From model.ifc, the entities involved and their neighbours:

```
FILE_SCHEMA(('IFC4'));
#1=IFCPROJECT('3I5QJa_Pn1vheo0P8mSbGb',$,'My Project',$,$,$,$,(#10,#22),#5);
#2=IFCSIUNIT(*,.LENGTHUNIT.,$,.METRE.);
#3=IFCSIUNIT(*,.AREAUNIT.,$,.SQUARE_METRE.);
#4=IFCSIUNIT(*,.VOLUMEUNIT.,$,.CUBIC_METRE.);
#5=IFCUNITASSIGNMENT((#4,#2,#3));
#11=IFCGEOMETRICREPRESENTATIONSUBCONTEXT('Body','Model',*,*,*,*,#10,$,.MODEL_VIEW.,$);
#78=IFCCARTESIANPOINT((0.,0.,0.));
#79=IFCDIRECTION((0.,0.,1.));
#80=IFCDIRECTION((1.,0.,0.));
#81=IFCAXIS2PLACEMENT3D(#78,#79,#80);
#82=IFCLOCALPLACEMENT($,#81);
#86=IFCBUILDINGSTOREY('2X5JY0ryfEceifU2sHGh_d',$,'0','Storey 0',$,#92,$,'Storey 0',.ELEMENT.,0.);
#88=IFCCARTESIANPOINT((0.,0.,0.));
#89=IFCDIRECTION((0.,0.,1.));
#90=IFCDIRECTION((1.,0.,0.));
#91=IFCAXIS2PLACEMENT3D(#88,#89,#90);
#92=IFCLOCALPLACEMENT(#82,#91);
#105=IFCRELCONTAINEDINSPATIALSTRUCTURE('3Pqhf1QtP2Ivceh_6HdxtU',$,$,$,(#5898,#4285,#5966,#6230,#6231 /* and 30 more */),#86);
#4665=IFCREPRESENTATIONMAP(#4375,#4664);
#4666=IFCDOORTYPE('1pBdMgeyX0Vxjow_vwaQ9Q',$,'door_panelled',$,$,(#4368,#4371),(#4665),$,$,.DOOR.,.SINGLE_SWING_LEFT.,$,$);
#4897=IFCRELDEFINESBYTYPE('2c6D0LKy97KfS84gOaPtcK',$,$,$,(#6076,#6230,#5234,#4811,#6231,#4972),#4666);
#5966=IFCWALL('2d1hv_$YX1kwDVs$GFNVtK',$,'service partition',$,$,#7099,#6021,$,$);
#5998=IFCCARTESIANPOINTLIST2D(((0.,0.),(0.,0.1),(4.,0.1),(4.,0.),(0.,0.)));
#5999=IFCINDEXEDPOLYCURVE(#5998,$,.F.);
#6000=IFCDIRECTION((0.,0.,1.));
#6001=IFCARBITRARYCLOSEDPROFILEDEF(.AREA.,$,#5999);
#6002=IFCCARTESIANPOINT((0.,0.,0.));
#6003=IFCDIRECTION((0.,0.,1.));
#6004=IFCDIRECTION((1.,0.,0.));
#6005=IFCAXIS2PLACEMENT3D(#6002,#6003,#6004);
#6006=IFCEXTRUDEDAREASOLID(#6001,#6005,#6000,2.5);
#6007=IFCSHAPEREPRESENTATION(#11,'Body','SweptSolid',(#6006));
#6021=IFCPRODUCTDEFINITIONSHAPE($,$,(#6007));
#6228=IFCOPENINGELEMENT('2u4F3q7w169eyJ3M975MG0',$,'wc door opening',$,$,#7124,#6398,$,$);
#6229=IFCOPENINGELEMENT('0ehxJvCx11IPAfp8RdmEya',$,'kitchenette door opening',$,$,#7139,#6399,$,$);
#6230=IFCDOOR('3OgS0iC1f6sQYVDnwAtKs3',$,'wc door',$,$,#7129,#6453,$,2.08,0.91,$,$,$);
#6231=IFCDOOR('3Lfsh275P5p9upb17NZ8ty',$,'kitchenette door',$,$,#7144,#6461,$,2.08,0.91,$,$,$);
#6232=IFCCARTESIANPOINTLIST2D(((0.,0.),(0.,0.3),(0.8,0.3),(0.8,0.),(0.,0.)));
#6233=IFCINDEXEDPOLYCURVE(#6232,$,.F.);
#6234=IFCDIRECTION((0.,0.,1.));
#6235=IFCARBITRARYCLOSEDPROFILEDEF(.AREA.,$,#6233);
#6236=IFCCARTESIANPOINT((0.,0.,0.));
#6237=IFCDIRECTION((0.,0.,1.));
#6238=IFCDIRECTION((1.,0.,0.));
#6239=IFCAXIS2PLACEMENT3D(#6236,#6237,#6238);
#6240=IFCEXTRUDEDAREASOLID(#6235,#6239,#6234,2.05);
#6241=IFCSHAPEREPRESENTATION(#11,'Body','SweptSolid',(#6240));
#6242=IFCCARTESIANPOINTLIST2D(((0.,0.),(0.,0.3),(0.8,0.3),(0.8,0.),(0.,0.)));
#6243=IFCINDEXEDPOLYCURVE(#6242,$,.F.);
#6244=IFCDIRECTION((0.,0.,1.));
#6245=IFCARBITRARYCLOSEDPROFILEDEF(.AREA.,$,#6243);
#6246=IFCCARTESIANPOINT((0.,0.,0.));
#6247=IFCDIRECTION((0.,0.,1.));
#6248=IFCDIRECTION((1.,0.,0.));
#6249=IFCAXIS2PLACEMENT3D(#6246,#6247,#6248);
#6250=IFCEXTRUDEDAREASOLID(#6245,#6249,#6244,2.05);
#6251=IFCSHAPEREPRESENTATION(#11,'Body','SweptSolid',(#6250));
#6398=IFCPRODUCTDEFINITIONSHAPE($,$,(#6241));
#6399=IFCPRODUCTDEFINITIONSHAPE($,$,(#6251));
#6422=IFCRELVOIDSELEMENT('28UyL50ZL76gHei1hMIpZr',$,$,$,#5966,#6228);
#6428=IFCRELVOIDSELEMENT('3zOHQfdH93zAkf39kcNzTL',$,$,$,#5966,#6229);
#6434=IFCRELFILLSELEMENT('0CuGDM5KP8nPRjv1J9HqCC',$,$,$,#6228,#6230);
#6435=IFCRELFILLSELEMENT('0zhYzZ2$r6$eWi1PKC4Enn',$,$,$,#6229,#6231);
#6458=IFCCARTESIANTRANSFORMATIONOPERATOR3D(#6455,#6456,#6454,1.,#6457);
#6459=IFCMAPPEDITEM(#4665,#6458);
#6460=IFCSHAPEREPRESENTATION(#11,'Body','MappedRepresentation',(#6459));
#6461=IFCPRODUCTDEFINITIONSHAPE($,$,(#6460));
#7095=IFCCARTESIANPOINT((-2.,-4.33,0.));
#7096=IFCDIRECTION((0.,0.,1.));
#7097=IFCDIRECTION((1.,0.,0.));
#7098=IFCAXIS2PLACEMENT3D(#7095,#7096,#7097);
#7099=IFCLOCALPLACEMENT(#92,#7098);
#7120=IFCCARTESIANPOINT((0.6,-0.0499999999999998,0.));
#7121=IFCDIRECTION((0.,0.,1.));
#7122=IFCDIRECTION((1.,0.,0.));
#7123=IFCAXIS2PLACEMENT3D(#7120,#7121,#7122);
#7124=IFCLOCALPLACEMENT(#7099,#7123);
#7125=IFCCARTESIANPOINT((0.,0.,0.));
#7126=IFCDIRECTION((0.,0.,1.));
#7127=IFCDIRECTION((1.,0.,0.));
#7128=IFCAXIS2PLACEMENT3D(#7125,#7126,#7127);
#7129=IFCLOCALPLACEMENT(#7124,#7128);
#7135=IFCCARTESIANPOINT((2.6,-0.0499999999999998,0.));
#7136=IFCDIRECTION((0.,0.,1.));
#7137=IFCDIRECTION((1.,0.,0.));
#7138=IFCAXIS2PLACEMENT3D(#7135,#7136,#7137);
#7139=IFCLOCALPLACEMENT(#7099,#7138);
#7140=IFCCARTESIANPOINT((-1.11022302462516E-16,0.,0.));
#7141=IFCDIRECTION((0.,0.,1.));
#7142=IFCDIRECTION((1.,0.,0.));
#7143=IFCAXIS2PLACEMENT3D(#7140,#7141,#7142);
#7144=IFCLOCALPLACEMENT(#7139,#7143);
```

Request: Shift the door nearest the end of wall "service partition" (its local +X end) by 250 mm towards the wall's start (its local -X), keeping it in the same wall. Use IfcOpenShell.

```python
import ifcopenshell
import ifcopenshell.api.geometry
import ifcopenshell.util.placement
import ifcopenshell.util.unit

model = ifcopenshell.open("model.ifc")
unit_scale = ifcopenshell.util.unit.calculate_unit_scale(model)

door = model.by_guid("3Lfsh275P5p9upb17NZ8ty")
opening = door.FillsVoids[0].RelatingOpeningElement
wall = opening.VoidsElements[0].RelatingBuildingElement

wall_matrix = ifcopenshell.util.placement.get_local_placement(wall.ObjectPlacement)
shift = wall_matrix[:3, 0] * -0.25 / unit_scale
before = ifcopenshell.util.placement.get_local_placement(door.ObjectPlacement)[:3, 3].copy()

# The door is placed relative to its opening, so it follows when the opening moves.
matrix = ifcopenshell.util.placement.get_local_placement(opening.ObjectPlacement)
matrix[:3, 3] += shift
ifcopenshell.api.geometry.edit_object_placement(
    model, product=opening, matrix=matrix, is_si=False, should_transform_children=True
)

after = ifcopenshell.util.placement.get_local_placement(door.ObjectPlacement)[:3, 3]
print("door moved by", (after - before).round(3) + 0.0)

model.write("model_rev.ifc")
```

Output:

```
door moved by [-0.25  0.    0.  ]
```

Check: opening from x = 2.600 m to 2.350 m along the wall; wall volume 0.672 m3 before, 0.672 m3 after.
